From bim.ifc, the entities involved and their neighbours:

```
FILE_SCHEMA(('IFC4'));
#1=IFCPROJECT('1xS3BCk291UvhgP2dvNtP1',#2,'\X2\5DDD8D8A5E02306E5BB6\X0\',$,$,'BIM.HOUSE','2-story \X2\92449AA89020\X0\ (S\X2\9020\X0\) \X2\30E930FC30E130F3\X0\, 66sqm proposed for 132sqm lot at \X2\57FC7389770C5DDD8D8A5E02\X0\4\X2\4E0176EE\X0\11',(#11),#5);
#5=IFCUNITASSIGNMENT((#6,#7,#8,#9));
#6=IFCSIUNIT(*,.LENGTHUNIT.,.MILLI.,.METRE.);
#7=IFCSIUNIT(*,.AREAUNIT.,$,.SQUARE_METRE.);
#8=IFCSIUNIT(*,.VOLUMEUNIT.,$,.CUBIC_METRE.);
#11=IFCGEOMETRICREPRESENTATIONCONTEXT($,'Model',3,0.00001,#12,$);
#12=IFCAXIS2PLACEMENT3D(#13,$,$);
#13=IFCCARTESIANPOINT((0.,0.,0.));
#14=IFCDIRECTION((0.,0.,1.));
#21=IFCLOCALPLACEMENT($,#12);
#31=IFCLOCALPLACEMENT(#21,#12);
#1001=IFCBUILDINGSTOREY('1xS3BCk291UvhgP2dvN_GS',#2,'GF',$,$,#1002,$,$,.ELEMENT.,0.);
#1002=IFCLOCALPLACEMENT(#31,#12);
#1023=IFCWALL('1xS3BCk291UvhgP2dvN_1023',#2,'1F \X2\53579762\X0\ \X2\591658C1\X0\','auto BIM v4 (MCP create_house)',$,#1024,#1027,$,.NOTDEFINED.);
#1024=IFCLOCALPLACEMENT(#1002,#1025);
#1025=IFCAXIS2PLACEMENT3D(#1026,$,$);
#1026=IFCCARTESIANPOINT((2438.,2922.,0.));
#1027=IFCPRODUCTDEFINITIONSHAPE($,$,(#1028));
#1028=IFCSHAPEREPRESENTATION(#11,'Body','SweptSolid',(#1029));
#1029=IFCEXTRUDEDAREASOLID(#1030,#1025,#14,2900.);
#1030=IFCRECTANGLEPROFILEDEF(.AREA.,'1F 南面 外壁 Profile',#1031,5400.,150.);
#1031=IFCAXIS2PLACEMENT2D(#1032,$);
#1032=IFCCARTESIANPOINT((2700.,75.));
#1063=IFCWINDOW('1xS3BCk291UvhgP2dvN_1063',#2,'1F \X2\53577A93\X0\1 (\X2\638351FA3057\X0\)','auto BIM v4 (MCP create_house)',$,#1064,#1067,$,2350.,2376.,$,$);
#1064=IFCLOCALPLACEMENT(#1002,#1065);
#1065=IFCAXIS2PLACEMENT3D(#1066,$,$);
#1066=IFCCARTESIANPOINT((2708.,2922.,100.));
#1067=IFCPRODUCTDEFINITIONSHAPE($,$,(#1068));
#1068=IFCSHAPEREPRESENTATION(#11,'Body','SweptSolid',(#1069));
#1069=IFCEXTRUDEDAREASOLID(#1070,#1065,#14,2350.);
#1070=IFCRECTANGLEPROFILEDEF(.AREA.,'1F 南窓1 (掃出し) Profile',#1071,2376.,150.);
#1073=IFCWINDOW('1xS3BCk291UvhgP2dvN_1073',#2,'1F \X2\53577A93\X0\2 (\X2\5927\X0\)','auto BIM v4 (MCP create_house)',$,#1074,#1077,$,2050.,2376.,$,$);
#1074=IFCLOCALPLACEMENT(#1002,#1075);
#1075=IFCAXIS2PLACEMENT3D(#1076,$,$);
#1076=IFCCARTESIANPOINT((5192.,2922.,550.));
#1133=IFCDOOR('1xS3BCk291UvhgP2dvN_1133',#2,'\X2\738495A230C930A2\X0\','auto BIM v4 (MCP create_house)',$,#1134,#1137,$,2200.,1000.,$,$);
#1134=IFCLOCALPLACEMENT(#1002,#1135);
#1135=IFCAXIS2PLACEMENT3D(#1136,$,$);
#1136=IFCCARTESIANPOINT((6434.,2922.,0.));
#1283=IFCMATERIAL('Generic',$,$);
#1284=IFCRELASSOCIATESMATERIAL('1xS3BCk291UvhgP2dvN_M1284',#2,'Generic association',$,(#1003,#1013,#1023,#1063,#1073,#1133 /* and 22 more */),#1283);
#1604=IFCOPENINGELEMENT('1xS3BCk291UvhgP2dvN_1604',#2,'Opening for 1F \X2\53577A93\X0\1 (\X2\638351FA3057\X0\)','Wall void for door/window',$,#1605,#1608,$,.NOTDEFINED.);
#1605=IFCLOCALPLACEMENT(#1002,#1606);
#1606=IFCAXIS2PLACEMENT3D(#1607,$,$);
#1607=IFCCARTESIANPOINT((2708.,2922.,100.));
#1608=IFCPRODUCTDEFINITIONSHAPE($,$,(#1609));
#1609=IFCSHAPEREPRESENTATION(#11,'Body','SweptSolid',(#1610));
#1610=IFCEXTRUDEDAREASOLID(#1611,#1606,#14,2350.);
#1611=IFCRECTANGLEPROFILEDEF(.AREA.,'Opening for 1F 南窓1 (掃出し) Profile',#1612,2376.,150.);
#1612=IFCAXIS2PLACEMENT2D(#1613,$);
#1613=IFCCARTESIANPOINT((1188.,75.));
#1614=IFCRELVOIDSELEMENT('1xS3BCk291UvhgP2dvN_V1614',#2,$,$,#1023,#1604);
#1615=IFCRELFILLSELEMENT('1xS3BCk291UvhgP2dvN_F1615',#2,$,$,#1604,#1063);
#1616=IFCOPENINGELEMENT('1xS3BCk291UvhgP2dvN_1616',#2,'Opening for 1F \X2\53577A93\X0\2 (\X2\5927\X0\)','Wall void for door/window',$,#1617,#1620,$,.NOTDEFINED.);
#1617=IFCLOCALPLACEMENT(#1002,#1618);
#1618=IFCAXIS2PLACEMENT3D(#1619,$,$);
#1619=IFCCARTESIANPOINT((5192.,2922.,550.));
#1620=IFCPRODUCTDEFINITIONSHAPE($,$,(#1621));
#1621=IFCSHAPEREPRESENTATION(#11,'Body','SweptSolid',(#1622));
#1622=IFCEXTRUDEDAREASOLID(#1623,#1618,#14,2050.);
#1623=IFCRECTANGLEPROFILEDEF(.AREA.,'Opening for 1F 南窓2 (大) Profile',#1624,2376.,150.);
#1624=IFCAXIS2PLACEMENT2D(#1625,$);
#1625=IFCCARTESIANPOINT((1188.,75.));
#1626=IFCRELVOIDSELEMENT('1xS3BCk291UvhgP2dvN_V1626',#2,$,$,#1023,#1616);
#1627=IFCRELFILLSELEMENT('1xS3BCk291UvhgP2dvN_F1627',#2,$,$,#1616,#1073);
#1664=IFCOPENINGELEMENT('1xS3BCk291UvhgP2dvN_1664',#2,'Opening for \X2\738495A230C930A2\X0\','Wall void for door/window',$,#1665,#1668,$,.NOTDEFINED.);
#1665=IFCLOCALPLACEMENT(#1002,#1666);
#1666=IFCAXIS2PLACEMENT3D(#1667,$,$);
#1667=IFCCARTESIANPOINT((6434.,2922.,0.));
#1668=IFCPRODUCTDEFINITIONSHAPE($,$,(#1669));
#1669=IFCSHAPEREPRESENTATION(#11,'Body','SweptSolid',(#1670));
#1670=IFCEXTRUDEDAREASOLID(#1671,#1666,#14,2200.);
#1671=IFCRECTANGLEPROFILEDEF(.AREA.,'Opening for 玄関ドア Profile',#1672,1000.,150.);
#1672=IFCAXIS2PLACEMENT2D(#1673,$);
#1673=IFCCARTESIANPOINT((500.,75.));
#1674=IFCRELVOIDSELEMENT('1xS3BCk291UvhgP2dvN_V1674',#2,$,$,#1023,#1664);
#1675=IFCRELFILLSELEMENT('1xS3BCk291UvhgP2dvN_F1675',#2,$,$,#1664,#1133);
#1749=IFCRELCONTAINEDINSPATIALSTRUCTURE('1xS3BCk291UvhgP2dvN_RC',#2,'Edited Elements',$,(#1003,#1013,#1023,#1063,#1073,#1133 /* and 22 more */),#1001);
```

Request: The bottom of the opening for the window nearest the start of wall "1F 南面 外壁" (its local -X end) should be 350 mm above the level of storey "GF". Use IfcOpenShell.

```python
import numpy as np
import ifcopenshell
import ifcopenshell.api.geometry
import ifcopenshell.geom
import ifcopenshell.util.element
import ifcopenshell.util.placement
import ifcopenshell.util.shape
import ifcopenshell.util.unit

model = ifcopenshell.open("bim.ifc")
unit_scale = ifcopenshell.util.unit.calculate_unit_scale(model)

window = model.by_guid("1xS3BCk291UvhgP2dvN_1063")
opening = window.FillsVoids[0].RelatingOpeningElement
storey = ifcopenshell.util.element.get_container(window, ifc_class="IfcBuildingStorey")
level = ifcopenshell.util.placement.get_local_placement(storey.ObjectPlacement)[2, 3]

# The opening's origin need not be at the sill, so measure its lowest point.
shape = ifcopenshell.geom.create_shape(ifcopenshell.geom.settings(), opening)
bottom = ifcopenshell.util.shape.get_shape_bottom_elevation(shape, shape.geometry) / unit_scale
dz = level + 0.35 / unit_scale - bottom

shift = np.array([0.0, 0.0, dz])
# The window is not placed relative to its opening, so move both.
for product in (opening, window):
    matrix = ifcopenshell.util.placement.get_local_placement(product.ObjectPlacement)
    matrix[:3, 3] += shift
    ifcopenshell.api.geometry.edit_object_placement(model, product=product, matrix=matrix, is_si=False)

print(f"moved by {dz * unit_scale:+.3f} m")

model.write("bim_edited.ifc")
```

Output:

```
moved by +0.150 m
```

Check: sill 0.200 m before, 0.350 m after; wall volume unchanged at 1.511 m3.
